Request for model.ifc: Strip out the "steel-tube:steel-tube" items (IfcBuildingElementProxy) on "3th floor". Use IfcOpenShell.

First a look at what the model holds.

```python
import ifcopenshell
import ifcopenshell.util.element

model = ifcopenshell.open("model.ifc")
print(model.schema)
storey = next(s for s in model.by_type("IfcBuildingStorey") if s.Name == "3th floor")
proxies = [e for e in ifcopenshell.util.element.get_decomposition(storey) if e.is_a("IfcBuildingElementProxy")]
seen = {}
for e in proxies:
    element_type = ifcopenshell.util.element.get_type(e)
    name = element_type.Name if element_type not in (None, e) else None
    seen[name] = seen.get(name, 0) + 1
for name, count in sorted(seen.items(), key=str):
    print(count, "x", name)
```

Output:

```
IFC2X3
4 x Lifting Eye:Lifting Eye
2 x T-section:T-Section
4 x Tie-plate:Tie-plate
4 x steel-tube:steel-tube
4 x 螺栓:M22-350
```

```python
import ifcopenshell
import ifcopenshell.api.root
import ifcopenshell.util.element

model = ifcopenshell.open("model.ifc")

storey = next(s for s in model.by_type("IfcBuildingStorey") if s.Name == "3th floor")
proxies = [e for e in ifcopenshell.util.element.get_decomposition(storey) if e.is_a("IfcBuildingElementProxy")]
targets = [e for e in proxies if (t := ifcopenshell.util.element.get_type(e)) not in (None, e) and t.Name == "steel-tube:steel-tube"]

for e in targets:
    ifcopenshell.api.root.remove_product(model, product=e)
print(len(targets), "removed")

model.write("model_edited.ifc")
```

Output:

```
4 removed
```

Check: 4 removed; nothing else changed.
